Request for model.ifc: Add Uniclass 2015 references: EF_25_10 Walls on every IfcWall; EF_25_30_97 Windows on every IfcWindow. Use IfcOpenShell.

First a look at what the model holds.

```python
import ifcopenshell

model = ifcopenshell.open("model.ifc")
print(model.schema)
print("classifications:", [c.Name for c in model.by_type("IfcClassification")])
for ifc_class in ("IfcDoor", "IfcRoof", "IfcStair", "IfcWall", "IfcWindow"):
    print(ifc_class, len(model.by_type(ifc_class)))
```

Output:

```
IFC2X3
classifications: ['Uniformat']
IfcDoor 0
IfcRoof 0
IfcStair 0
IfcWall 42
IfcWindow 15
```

```python
import ifcopenshell
import ifcopenshell.api.classification

model = ifcopenshell.open("model.ifc")

# IFC2X3 requires Source and Edition and has no link from the project to the system.
system = model.create_entity("IfcClassification", Source="NBS", Edition="2015", Name="Uniclass 2015")

codes = {
    "IfcWall": ("EF_25_10", "Walls"),
    "IfcWindow": ("EF_25_30_97", "Windows"),
}
for ifc_class, (code, name) in codes.items():
    products = model.by_type(ifc_class)
    ifcopenshell.api.classification.add_reference(
        model, products=products, classification=system, identification=code, name=name
    )
    print(code, len(products))

model.write("model-out.ifc")
```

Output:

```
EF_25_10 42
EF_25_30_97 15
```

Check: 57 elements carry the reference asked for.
